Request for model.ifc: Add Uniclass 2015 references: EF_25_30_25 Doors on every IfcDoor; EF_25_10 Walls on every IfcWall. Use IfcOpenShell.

First a look at what the model holds.

```python
import ifcopenshell

model = ifcopenshell.open("model.ifc")
print(model.schema)
print("classifications:", [c.Name for c in model.by_type("IfcClassification")])
for ifc_class in ("IfcDoor", "IfcRoof", "IfcStair", "IfcWall", "IfcWindow"):
    print(ifc_class, len(model.by_type(ifc_class)))
```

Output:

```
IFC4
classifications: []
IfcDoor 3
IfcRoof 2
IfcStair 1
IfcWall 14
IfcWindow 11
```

```python
import ifcopenshell
import ifcopenshell.api.classification

model = ifcopenshell.open("model.ifc")

system = ifcopenshell.api.classification.add_classification(model, classification="Uniclass 2015")

codes = {
    "IfcDoor": ("EF_25_30_25", "Doors"),
    "IfcWall": ("EF_25_10", "Walls"),
}
for ifc_class, (code, name) in codes.items():
    products = model.by_type(ifc_class)
    ifcopenshell.api.classification.add_reference(
        model, products=products, classification=system, identification=code, name=name
    )
    print(code, len(products))

model.write("model-out.ifc")
```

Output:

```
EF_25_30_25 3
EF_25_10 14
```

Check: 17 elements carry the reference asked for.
